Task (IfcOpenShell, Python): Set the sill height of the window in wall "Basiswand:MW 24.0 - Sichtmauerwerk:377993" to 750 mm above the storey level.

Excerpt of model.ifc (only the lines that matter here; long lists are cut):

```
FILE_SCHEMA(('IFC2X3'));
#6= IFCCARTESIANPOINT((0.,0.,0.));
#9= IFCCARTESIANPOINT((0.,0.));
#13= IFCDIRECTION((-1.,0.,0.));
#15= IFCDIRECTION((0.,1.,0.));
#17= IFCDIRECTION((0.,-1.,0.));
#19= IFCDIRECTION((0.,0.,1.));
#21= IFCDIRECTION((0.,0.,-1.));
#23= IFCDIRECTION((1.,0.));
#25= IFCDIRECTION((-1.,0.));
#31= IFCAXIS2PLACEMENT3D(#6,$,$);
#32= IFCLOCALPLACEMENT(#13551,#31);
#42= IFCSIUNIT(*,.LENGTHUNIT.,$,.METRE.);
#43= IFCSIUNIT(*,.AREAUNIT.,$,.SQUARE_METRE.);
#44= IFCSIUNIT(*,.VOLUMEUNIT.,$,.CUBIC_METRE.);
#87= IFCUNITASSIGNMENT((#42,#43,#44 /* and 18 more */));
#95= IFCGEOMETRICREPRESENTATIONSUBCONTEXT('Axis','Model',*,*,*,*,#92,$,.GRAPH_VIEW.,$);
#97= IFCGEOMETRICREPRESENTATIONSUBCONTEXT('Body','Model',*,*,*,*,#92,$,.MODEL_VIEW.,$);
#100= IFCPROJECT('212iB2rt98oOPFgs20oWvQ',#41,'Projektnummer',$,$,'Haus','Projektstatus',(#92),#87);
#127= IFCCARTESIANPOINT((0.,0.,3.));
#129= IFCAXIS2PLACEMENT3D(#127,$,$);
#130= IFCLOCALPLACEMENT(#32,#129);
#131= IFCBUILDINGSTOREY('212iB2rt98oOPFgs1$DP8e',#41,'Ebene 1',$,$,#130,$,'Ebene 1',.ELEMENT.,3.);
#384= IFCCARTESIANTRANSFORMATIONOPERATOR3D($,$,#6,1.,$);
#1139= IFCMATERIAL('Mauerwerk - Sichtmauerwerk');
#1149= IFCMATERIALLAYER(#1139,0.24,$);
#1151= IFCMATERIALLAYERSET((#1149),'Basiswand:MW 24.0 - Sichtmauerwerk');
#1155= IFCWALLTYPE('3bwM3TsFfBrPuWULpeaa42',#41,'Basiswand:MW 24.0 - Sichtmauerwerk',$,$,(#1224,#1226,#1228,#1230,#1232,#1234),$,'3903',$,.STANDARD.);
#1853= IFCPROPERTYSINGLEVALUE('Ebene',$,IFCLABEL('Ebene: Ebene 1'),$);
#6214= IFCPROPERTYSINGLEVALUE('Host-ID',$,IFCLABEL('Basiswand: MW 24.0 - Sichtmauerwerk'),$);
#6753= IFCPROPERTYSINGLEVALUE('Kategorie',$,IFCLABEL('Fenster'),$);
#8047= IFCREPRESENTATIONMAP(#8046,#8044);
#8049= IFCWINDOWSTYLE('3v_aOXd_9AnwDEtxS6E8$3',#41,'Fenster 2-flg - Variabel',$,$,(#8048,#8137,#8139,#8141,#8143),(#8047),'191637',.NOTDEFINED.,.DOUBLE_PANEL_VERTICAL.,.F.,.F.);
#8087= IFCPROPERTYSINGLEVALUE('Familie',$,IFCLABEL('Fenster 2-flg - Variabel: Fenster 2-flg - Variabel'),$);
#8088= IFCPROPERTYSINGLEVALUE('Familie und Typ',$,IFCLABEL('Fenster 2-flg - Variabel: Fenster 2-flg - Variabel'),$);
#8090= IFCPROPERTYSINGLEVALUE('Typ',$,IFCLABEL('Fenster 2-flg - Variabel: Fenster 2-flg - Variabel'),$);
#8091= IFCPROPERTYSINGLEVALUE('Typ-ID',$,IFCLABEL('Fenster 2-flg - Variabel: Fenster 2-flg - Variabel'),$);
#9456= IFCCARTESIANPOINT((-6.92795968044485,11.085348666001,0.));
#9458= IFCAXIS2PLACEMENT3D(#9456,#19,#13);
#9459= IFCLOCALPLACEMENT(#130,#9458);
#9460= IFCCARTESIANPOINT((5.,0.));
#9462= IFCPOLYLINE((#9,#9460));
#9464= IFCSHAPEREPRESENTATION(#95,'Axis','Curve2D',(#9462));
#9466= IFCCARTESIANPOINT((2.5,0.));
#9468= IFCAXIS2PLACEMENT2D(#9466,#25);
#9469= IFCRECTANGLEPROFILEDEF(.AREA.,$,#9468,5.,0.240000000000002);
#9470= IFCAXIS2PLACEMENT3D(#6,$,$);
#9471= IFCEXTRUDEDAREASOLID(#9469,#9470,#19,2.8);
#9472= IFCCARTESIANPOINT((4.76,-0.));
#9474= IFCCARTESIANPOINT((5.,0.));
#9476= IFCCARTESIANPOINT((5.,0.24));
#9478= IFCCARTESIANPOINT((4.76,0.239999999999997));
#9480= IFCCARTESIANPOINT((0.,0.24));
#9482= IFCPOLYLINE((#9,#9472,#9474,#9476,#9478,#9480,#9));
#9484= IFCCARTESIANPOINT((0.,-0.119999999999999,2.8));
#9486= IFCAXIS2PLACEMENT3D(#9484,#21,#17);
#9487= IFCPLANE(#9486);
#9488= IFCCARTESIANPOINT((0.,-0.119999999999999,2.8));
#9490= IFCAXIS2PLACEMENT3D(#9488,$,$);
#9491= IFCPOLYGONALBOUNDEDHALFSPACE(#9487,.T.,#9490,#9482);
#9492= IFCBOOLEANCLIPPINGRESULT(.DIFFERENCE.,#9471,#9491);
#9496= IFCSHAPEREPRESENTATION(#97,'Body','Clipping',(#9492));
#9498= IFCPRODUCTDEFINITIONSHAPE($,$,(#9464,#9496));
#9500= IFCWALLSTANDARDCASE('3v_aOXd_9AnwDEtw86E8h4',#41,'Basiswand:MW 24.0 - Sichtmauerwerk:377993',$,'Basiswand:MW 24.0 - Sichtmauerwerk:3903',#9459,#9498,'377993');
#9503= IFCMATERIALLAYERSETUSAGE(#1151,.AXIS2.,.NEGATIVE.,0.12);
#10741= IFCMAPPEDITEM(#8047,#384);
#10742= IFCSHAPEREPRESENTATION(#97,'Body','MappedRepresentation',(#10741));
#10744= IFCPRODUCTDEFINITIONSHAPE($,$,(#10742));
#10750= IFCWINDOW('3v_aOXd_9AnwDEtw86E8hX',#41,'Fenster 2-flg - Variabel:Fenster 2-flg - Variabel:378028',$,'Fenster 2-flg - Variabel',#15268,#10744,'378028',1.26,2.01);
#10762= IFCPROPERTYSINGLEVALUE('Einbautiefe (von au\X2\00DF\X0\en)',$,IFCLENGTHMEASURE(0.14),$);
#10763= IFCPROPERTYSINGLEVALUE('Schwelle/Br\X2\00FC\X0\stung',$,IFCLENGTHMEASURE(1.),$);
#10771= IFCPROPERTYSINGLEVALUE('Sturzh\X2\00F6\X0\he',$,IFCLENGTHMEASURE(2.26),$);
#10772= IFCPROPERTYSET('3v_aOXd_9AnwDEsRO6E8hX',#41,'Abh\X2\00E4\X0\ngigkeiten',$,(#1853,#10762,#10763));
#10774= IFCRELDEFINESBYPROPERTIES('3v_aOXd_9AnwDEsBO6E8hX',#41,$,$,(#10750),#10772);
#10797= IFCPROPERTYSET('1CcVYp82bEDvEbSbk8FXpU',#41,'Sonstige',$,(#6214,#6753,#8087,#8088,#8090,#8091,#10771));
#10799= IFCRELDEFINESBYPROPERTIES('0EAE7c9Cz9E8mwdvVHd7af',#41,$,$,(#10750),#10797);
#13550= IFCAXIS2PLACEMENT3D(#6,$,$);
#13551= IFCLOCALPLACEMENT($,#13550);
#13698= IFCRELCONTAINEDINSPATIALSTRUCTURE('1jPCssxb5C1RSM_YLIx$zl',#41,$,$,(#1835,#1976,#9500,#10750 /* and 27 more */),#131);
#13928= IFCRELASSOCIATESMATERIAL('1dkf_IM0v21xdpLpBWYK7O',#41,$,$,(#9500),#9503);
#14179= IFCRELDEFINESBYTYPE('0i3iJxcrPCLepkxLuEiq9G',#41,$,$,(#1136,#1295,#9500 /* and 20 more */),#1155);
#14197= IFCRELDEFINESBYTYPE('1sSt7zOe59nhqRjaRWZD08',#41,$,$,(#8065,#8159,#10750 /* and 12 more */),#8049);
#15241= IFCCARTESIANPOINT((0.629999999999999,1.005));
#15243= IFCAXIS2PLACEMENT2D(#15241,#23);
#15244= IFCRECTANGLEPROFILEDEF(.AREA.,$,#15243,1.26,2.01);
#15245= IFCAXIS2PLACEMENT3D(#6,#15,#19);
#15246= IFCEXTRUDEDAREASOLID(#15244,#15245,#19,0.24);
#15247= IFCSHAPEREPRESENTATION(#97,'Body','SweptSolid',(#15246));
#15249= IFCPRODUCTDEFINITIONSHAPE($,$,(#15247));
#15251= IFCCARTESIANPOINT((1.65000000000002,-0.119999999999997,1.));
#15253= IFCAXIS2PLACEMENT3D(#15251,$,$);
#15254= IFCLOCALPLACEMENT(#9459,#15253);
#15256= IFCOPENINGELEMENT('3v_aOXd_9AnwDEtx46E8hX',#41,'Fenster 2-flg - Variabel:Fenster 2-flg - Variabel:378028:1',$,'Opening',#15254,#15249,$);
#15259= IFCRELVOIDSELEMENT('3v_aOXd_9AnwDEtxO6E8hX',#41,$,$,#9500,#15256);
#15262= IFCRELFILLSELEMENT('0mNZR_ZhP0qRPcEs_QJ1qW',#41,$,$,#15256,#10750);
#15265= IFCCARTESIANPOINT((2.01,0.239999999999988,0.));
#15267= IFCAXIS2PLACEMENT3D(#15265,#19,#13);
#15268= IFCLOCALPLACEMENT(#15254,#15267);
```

```python
import numpy as np
import ifcopenshell
import ifcopenshell.api.geometry
import ifcopenshell.api.pset
import ifcopenshell.geom
import ifcopenshell.util.element
import ifcopenshell.util.placement
import ifcopenshell.util.shape
import ifcopenshell.util.unit

model = ifcopenshell.open("model.ifc")
unit_scale = ifcopenshell.util.unit.calculate_unit_scale(model)

window = model.by_guid("3v_aOXd_9AnwDEtw86E8hX")
opening = window.FillsVoids[0].RelatingOpeningElement
storey = ifcopenshell.util.element.get_container(window, ifc_class="IfcBuildingStorey")
level = ifcopenshell.util.placement.get_local_placement(storey.ObjectPlacement)[2, 3]

# The opening's origin need not be at the sill, so measure its lowest point.
shape = ifcopenshell.geom.create_shape(ifcopenshell.geom.settings(), opening)
bottom = ifcopenshell.util.shape.get_shape_bottom_elevation(shape, shape.geometry) / unit_scale
dz = level + 0.75 / unit_scale - bottom

shift = np.array([0.0, 0.0, dz])
# The window is placed relative to its opening, so it follows when the opening moves.
matrix = ifcopenshell.util.placement.get_local_placement(opening.ObjectPlacement)
matrix[:3, 3] += shift
ifcopenshell.api.geometry.edit_object_placement(
    model, product=opening, matrix=matrix, is_si=False, should_transform_children=True
)

# Keep the stored heights in step.
pset = model.by_id(ifcopenshell.util.element.get_pset(window, "Abhängigkeiten", should_inherit=False)["id"])
ifcopenshell.api.pset.edit_pset(model, pset=pset, properties={
    "Schwelle/Brüstung": model.create_entity("IfcLengthMeasure", ifcopenshell.util.element.get_pset(window, "Abhängigkeiten", "Schwelle/Brüstung") + dz),
})
pset = model.by_id(ifcopenshell.util.element.get_pset(window, "Sonstige", should_inherit=False)["id"])
ifcopenshell.api.pset.edit_pset(model, pset=pset, properties={
    "Sturzhöhe": model.create_entity("IfcLengthMeasure", ifcopenshell.util.element.get_pset(window, "Sonstige", "Sturzhöhe") + dz),
})

print(f"moved by {dz * unit_scale:+.3f} m")

model.write("model_rev.ifc")
```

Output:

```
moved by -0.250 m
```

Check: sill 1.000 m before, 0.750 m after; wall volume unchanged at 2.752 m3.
